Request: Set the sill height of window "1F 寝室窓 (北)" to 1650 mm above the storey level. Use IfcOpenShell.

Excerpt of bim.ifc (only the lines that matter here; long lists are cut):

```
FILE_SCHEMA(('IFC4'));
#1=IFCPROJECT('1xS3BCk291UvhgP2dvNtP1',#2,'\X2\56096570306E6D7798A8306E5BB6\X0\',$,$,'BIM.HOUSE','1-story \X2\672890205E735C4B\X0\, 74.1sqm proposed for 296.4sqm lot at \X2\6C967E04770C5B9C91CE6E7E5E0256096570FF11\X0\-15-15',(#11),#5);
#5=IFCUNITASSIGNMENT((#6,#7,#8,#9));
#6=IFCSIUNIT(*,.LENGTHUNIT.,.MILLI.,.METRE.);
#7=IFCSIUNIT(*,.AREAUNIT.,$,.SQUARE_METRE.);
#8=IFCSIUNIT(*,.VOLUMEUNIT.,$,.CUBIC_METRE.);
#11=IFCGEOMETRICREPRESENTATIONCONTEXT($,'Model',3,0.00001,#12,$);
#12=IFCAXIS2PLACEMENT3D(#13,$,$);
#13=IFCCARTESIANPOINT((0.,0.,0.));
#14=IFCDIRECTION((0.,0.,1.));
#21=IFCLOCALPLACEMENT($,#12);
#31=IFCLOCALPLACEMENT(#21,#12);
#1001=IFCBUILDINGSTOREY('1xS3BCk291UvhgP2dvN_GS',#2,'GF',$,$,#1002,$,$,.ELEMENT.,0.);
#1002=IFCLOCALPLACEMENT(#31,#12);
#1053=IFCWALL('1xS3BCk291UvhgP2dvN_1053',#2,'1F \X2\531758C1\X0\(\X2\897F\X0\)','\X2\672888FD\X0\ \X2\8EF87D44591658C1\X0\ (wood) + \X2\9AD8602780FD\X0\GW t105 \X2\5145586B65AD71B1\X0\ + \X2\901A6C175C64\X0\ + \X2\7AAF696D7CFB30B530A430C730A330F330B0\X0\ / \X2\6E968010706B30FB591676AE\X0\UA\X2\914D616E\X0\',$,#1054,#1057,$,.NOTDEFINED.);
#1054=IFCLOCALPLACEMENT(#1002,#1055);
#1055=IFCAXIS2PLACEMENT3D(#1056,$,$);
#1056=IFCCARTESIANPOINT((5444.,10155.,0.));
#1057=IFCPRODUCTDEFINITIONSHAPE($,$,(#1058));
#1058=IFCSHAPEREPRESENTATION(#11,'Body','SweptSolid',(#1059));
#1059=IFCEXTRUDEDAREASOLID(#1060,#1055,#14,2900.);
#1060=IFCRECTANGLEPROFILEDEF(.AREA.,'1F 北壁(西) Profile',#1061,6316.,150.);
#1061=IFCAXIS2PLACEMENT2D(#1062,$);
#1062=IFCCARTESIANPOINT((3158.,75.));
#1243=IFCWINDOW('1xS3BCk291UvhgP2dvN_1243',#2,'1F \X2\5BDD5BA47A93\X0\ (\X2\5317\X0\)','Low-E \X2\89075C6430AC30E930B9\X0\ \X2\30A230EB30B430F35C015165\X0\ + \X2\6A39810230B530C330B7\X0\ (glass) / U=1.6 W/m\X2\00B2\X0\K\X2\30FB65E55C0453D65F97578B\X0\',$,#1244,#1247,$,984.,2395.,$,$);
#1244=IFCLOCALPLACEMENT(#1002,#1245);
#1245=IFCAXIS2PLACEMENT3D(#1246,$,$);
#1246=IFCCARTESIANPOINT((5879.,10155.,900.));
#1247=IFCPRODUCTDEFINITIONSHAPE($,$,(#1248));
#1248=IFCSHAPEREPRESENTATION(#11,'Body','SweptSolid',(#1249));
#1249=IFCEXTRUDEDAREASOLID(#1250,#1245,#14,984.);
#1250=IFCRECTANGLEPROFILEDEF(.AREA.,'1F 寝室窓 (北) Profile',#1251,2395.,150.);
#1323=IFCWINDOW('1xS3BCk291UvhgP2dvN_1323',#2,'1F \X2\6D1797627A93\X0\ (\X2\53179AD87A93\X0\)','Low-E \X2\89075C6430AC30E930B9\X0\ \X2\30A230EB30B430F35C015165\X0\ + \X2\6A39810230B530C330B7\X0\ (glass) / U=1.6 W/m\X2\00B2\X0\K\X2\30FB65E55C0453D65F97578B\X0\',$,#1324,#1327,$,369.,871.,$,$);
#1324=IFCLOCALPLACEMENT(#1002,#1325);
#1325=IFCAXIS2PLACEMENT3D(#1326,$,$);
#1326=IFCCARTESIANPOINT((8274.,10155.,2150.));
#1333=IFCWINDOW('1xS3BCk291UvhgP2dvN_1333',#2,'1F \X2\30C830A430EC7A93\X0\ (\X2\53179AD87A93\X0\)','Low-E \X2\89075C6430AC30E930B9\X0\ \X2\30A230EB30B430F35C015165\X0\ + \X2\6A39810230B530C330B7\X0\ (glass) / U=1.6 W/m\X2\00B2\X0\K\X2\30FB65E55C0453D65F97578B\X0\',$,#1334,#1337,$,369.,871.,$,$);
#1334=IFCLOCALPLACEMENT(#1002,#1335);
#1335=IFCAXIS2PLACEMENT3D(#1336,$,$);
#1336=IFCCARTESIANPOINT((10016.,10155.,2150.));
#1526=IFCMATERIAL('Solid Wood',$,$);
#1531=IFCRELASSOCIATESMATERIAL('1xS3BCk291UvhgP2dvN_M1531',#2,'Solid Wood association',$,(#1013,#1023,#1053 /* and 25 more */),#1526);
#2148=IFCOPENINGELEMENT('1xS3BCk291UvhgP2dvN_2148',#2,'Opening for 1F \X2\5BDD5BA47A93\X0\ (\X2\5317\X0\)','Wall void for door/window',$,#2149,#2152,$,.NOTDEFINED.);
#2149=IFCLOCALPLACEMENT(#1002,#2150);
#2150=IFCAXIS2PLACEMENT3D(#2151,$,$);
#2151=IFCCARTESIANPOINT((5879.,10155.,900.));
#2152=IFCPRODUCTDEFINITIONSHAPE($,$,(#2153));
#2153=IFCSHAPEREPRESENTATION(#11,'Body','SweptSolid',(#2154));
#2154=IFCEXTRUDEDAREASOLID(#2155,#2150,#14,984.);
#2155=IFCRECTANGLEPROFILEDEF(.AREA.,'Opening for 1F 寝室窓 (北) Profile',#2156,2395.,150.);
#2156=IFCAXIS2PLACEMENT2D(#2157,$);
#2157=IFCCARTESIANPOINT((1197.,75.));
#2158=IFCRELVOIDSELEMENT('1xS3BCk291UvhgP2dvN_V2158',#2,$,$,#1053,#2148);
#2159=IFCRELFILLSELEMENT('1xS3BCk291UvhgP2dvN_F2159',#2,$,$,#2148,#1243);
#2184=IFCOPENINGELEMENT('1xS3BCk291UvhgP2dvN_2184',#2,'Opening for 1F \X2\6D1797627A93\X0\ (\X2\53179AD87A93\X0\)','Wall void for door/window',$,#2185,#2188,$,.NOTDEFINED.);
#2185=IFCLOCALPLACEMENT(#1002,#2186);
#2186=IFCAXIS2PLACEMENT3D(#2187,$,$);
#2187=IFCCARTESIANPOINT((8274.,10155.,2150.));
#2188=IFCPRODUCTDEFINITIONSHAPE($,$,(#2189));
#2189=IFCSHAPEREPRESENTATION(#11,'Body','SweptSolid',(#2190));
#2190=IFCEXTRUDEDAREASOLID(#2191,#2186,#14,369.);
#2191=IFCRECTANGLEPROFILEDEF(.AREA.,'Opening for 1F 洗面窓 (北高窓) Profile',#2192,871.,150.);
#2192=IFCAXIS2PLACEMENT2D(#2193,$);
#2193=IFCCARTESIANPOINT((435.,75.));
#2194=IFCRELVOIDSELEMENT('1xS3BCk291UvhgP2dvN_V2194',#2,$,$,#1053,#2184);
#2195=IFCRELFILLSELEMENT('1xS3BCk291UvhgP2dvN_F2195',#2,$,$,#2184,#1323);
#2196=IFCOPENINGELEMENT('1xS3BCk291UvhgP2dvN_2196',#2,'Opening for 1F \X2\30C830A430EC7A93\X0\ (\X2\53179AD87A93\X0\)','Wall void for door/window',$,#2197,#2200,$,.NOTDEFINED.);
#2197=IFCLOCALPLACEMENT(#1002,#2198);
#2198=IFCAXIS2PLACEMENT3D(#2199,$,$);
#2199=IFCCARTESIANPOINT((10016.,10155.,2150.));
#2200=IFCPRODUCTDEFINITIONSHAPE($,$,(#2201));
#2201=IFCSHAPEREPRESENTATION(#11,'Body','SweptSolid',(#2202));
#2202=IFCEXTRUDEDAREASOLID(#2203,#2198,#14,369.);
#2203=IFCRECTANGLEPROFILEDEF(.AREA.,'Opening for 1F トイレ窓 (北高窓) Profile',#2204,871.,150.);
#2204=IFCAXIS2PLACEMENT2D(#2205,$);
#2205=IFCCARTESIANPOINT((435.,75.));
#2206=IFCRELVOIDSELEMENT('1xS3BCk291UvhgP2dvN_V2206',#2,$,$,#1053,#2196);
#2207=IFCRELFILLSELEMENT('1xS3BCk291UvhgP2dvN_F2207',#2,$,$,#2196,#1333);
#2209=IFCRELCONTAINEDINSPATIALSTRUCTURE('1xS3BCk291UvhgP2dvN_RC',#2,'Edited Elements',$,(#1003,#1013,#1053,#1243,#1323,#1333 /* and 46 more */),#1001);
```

```python
import numpy as np
import ifcopenshell
import ifcopenshell.api.geometry
import ifcopenshell.geom
import ifcopenshell.util.element
import ifcopenshell.util.placement
import ifcopenshell.util.shape
import ifcopenshell.util.unit

model = ifcopenshell.open("bim.ifc")
unit_scale = ifcopenshell.util.unit.calculate_unit_scale(model)

window = model.by_guid("1xS3BCk291UvhgP2dvN_1243")
opening = window.FillsVoids[0].RelatingOpeningElement
storey = ifcopenshell.util.element.get_container(window, ifc_class="IfcBuildingStorey")
level = ifcopenshell.util.placement.get_local_placement(storey.ObjectPlacement)[2, 3]

# The opening's origin need not be at the sill, so measure its lowest point.
shape = ifcopenshell.geom.create_shape(ifcopenshell.geom.settings(), opening)
bottom = ifcopenshell.util.shape.get_shape_bottom_elevation(shape, shape.geometry) / unit_scale
dz = level + 1.65 / unit_scale - bottom

shift = np.array([0.0, 0.0, dz])
# The window is not placed relative to its opening, so move both.
for product in (opening, window):
    matrix = ifcopenshell.util.placement.get_local_placement(product.ObjectPlacement)
    matrix[:3, 3] += shift
    ifcopenshell.api.geometry.edit_object_placement(model, product=product, matrix=matrix, is_si=False)

print(f"moved by {dz * unit_scale:+.3f} m")

model.write("bim_rev.ifc")
```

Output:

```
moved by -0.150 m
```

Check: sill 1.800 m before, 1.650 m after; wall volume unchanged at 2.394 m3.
